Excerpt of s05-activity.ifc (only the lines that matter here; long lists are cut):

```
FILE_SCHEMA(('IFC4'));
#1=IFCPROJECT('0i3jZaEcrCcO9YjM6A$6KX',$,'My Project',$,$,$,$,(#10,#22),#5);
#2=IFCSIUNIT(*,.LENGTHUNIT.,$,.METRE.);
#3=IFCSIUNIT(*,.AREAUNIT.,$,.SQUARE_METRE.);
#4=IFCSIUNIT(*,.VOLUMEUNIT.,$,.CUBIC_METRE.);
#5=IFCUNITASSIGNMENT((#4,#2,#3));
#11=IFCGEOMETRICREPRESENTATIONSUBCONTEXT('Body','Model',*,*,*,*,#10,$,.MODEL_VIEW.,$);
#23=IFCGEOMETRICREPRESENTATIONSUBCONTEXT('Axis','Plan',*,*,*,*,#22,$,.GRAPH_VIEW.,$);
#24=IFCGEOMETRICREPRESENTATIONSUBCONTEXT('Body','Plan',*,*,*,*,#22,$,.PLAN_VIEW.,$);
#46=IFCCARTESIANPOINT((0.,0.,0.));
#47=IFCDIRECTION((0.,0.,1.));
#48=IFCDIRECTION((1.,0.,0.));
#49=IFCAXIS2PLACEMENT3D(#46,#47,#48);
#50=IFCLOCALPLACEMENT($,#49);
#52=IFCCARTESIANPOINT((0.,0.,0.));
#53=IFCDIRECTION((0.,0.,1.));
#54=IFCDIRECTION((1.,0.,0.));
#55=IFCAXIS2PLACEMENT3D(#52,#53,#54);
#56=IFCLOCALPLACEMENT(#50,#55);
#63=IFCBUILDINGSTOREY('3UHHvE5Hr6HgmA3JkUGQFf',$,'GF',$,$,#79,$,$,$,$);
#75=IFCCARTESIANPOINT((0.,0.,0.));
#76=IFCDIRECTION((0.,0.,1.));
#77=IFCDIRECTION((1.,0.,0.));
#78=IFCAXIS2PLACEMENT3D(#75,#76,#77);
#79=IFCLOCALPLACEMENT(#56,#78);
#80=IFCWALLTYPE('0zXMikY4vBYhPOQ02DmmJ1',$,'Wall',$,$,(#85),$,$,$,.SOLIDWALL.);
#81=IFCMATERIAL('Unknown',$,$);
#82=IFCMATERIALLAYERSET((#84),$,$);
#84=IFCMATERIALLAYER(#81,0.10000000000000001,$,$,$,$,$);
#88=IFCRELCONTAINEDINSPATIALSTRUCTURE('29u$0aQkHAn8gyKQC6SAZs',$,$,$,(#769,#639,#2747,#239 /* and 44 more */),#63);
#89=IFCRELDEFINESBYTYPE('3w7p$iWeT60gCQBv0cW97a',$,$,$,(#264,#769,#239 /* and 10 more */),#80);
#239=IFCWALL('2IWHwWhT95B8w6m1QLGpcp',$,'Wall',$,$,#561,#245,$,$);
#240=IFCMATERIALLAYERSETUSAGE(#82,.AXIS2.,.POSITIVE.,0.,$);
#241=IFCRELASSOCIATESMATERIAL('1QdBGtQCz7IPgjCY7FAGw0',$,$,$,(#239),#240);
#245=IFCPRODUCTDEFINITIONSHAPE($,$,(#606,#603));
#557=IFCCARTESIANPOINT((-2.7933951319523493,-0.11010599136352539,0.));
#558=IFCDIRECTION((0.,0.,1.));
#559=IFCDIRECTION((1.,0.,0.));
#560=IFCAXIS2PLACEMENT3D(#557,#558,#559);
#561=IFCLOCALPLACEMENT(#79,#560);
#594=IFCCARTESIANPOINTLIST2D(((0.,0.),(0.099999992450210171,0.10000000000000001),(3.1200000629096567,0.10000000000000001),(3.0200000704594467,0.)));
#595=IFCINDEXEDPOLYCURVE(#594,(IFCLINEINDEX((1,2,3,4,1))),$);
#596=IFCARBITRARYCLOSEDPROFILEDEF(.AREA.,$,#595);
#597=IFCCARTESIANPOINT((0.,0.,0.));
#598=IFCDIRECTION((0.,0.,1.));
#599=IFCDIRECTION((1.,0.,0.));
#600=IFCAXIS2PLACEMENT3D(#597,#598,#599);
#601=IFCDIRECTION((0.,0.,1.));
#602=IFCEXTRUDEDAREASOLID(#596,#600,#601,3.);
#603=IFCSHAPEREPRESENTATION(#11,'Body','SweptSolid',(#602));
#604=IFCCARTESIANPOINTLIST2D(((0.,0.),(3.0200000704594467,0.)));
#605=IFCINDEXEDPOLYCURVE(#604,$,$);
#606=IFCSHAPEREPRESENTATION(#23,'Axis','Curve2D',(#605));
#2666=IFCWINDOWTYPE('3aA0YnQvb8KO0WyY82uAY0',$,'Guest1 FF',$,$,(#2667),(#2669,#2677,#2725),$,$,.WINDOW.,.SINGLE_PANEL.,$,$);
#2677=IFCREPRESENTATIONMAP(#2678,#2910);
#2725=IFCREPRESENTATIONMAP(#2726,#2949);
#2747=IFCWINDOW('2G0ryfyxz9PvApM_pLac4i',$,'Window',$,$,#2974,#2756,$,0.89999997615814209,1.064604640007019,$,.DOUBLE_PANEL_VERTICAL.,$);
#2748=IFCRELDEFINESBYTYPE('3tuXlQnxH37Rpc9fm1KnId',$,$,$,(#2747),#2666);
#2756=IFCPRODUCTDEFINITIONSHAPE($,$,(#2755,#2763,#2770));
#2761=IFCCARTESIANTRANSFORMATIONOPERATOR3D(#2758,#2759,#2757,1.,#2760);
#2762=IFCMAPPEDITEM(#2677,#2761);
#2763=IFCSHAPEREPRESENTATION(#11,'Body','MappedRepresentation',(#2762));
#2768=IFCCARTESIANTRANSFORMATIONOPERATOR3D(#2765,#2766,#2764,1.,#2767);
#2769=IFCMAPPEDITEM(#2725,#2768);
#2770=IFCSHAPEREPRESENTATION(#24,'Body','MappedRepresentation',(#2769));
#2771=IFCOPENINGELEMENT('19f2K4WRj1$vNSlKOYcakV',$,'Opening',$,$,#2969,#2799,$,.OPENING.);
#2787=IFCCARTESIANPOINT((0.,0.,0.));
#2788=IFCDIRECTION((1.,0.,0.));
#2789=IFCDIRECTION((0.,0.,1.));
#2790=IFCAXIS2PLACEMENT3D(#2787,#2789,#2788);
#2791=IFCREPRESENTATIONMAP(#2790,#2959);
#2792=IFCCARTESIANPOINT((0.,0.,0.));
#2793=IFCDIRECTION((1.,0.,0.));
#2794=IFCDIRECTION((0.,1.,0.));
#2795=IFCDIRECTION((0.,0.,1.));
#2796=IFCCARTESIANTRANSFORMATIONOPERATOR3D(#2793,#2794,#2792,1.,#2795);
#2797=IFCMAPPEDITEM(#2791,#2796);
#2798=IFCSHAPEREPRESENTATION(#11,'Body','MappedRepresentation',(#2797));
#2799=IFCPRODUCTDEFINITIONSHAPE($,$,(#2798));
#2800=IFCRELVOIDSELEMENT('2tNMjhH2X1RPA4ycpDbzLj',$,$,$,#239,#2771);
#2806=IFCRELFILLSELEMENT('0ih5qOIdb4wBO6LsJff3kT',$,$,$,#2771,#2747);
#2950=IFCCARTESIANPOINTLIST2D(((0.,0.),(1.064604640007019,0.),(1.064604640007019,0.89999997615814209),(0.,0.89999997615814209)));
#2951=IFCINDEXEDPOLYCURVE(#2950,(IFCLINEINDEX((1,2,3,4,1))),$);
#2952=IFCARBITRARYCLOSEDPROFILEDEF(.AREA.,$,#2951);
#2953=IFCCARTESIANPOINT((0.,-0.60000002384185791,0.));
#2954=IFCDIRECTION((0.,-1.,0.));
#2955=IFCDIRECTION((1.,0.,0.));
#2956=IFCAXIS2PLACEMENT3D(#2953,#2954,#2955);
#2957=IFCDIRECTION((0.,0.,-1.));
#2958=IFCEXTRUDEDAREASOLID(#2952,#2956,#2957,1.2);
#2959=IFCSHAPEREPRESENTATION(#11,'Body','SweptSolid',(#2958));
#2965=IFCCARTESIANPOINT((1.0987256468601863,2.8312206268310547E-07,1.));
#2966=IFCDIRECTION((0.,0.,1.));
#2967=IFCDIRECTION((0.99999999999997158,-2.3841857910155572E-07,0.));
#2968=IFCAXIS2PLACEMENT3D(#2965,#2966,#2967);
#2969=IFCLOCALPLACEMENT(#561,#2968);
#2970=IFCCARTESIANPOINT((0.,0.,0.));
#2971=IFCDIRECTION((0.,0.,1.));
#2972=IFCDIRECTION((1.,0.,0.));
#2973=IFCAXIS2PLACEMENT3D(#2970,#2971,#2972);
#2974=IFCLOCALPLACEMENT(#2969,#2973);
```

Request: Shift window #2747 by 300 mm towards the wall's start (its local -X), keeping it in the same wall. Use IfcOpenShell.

```python
import ifcopenshell
import ifcopenshell.api.geometry
import ifcopenshell.util.placement

model = ifcopenshell.open("s05-activity.ifc")

window = model.by_guid("2G0ryfyxz9PvApM_pLac4i")
opening = window.FillsVoids[0].RelatingOpeningElement
wall = opening.VoidsElements[0].RelatingBuildingElement

wall_matrix = ifcopenshell.util.placement.get_local_placement(wall.ObjectPlacement)
shift = wall_matrix[:3, 0] * -0.3
before = ifcopenshell.util.placement.get_local_placement(window.ObjectPlacement)[:3, 3].copy()

# The window is placed relative to its opening, so it follows when the opening moves.
matrix = ifcopenshell.util.placement.get_local_placement(opening.ObjectPlacement)
matrix[:3, 3] += shift
ifcopenshell.api.geometry.edit_object_placement(
    model, product=opening, matrix=matrix, is_si=False, should_transform_children=True
)

after = ifcopenshell.util.placement.get_local_placement(window.ObjectPlacement)[:3, 3]
print("window moved by", (after - before).round(3) + 0.0)

model.write("s05-activity_updated.ifc")
```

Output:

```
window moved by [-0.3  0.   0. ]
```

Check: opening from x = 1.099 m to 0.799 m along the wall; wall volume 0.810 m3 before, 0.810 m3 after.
